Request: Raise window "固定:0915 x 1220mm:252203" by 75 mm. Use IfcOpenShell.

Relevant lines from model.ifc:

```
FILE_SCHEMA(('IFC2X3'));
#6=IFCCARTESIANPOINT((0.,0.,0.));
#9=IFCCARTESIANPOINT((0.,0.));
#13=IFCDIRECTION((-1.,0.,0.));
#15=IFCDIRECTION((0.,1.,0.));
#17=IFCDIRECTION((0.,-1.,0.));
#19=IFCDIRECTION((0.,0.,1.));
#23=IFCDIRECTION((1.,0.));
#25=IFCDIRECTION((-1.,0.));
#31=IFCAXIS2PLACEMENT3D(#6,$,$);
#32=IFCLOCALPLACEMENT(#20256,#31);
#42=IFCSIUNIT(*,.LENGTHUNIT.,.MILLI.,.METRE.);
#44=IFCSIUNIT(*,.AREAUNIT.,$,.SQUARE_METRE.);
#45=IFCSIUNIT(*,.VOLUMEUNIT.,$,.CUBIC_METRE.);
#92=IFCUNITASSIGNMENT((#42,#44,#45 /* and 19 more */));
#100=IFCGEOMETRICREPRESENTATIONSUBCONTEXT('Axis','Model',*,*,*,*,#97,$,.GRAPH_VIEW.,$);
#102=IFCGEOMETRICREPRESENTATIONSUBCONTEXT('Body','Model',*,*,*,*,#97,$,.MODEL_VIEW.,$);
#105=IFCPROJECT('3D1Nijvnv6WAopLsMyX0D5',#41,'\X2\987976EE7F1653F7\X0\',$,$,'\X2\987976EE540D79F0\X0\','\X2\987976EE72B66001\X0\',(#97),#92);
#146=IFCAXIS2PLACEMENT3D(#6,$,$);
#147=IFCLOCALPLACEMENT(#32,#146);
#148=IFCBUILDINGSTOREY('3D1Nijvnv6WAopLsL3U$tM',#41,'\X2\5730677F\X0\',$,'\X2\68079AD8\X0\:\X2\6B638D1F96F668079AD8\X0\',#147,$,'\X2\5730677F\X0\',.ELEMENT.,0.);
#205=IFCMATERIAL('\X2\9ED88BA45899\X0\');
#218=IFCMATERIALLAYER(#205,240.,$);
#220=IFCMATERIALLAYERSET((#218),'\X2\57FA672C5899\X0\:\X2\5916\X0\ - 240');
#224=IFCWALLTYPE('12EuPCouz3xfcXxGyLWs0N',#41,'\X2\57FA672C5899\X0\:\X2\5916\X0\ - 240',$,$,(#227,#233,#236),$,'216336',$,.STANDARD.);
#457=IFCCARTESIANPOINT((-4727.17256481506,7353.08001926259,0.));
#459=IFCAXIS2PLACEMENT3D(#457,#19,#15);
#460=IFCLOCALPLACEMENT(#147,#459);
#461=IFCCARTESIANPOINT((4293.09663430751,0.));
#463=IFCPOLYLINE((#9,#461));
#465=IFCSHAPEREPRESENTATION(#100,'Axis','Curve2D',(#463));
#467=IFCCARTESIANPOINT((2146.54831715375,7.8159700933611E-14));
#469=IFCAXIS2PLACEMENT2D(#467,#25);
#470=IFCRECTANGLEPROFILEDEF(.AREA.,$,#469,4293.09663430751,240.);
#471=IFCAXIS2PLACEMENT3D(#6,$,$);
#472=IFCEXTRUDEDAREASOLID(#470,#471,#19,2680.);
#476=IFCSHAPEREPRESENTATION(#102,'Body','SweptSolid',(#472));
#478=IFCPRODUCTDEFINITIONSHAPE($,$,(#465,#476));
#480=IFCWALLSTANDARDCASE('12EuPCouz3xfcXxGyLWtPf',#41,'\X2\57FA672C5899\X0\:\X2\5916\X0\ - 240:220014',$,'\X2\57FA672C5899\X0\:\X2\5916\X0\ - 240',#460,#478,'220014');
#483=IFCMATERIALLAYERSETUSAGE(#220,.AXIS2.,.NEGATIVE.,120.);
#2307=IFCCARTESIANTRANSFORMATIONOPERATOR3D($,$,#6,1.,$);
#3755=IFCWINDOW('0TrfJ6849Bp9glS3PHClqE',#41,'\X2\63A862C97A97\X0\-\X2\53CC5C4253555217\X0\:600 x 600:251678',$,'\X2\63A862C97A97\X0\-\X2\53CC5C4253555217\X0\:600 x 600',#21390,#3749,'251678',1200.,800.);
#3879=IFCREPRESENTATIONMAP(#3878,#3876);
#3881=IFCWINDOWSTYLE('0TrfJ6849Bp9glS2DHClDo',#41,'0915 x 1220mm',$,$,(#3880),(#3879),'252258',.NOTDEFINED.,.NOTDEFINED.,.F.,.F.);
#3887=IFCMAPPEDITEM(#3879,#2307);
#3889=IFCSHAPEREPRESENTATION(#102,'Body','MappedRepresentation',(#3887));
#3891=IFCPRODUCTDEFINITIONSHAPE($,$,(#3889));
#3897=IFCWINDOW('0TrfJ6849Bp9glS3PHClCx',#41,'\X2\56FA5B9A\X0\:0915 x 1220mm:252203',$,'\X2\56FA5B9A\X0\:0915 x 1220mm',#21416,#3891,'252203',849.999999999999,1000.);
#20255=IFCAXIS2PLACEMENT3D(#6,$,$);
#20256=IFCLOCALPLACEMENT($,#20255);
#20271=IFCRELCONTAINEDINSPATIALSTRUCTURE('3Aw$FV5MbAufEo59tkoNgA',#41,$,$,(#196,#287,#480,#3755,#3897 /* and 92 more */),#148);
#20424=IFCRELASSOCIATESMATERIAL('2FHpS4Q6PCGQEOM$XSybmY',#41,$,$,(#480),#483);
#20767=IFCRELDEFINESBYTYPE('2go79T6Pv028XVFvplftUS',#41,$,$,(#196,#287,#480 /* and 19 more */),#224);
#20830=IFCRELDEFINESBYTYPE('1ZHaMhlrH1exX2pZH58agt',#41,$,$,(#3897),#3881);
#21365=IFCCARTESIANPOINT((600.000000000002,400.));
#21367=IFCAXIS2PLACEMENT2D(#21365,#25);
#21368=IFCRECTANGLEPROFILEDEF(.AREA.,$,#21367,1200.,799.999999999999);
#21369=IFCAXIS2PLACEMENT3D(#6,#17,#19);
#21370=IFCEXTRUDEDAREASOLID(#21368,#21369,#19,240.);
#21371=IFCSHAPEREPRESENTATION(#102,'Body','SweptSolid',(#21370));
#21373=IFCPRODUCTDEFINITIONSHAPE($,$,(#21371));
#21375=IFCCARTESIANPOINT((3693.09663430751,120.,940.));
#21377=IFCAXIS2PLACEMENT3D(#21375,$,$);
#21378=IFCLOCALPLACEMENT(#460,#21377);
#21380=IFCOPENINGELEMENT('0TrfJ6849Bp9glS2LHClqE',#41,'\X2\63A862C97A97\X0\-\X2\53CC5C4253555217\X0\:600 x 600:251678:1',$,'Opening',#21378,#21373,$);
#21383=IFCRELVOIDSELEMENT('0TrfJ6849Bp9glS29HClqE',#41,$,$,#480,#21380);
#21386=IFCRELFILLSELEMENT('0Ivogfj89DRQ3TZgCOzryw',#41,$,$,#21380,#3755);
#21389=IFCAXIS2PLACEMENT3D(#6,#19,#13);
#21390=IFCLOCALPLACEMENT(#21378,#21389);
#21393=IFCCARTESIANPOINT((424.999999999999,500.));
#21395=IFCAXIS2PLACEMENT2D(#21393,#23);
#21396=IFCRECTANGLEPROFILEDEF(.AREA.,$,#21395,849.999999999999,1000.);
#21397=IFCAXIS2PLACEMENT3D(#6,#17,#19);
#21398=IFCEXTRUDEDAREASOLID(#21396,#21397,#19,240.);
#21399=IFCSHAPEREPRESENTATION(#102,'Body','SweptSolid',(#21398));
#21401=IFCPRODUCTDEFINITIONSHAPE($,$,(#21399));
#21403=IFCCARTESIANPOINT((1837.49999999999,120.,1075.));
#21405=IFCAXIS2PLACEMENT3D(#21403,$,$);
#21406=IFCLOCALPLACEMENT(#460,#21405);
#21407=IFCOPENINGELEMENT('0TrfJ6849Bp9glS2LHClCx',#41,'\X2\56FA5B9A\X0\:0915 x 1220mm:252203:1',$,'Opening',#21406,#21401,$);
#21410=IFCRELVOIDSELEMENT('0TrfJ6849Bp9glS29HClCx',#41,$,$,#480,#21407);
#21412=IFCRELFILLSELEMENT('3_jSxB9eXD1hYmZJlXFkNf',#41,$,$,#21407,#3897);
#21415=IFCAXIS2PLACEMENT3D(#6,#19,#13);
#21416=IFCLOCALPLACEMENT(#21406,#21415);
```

```python
import numpy as np
import ifcopenshell
import ifcopenshell.api.geometry
import ifcopenshell.util.placement
import ifcopenshell.util.unit

model = ifcopenshell.open("model.ifc")
unit_scale = ifcopenshell.util.unit.calculate_unit_scale(model)

window = model.by_guid("0TrfJ6849Bp9glS3PHClCx")
opening = window.FillsVoids[0].RelatingOpeningElement
dz = 75.0

shift = np.array([0.0, 0.0, dz])
# The window is placed relative to its opening, so it follows when the opening moves.
matrix = ifcopenshell.util.placement.get_local_placement(opening.ObjectPlacement)
matrix[:3, 3] += shift
ifcopenshell.api.geometry.edit_object_placement(
    model, product=opening, matrix=matrix, is_si=False, should_transform_children=True
)

print(f"moved by {dz * unit_scale:+.3f} m")

model.write("model_v2.ifc")
```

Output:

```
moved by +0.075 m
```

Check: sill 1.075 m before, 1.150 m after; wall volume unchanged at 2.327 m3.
